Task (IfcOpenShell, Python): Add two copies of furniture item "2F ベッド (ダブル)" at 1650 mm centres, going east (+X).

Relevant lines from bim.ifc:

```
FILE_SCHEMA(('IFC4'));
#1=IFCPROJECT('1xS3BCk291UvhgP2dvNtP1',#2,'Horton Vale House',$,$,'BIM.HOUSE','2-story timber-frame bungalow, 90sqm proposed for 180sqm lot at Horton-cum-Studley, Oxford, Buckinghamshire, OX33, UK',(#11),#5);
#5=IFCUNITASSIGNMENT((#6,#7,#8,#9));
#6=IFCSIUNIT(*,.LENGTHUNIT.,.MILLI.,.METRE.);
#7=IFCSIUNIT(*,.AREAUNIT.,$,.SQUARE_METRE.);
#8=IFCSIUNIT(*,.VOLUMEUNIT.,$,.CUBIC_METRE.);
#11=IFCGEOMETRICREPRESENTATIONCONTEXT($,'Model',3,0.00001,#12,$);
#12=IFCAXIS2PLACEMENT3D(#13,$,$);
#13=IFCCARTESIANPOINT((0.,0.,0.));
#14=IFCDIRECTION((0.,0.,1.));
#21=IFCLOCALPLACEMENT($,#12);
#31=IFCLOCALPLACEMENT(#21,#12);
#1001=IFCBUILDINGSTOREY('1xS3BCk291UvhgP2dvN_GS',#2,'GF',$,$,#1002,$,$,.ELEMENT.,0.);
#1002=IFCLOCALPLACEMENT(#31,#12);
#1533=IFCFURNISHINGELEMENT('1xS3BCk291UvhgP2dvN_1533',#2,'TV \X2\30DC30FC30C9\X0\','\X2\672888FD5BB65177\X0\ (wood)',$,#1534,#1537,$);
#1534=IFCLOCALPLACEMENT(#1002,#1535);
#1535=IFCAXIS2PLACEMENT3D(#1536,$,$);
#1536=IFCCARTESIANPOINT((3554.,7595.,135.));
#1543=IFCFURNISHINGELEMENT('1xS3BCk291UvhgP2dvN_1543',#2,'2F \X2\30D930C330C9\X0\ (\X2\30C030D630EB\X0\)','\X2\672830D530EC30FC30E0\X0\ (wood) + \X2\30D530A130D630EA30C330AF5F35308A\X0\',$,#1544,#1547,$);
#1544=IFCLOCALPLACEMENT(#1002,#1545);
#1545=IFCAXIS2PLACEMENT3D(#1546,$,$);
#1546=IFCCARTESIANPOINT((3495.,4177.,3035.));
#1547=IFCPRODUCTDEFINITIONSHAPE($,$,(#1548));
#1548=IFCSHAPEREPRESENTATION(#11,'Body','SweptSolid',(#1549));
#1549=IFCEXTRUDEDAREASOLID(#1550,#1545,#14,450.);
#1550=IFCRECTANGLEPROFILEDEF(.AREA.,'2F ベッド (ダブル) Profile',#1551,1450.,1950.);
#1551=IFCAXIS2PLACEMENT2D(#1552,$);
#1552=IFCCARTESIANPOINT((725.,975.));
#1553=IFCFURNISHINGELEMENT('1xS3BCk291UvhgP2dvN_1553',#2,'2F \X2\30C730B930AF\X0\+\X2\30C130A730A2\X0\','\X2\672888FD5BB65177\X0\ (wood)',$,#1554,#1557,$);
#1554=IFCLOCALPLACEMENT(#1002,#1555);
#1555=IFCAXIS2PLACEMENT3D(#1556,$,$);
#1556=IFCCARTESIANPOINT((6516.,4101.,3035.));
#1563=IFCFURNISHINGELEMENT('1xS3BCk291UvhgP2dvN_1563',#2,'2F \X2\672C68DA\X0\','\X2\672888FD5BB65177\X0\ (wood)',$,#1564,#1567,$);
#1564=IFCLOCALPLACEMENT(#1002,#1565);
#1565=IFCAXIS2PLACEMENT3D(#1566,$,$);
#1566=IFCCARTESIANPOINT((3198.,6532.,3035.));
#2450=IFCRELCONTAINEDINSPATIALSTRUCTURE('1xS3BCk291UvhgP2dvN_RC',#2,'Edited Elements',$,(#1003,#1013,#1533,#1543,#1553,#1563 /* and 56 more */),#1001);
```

```python
import numpy as np
import ifcopenshell
import ifcopenshell.api.geometry
import ifcopenshell.api.root
import ifcopenshell.util.element
import ifcopenshell.util.placement

model = ifcopenshell.open("bim.ifc")


def reuse_history(source, copy):
    """copy_class also copies each property set's owner history, people and application; keep the originals."""
    for rel in copy.IsDefinedBy:
        if rel.is_a("IfcRelDefinesByProperties") and (history := rel.RelatingPropertyDefinition.OwnerHistory):
            rel.RelatingPropertyDefinition.OwnerHistory = source.OwnerHistory
            ifcopenshell.util.element.remove_deep2(model, history)


source = model.by_guid("1xS3BCk291UvhgP2dvN_1543")
base = ifcopenshell.util.placement.get_local_placement(source.ObjectPlacement)
step = np.array([1.0, 0.0, 0.0]) * 1650.0

for i in range(1, 3):
    copy = ifcopenshell.api.root.copy_class(model, product=source)
    copy.Representation = ifcopenshell.util.element.copy_deep(
        model, source.Representation, exclude=["IfcGeometricRepresentationContext", "IfcRepresentationMap"]
    )
    reuse_history(source, copy)
    matrix = base.copy()
    matrix[:3, 3] += i * step
    print("added at", matrix[:3, 3].round(3) + 0.0)
    ifcopenshell.api.geometry.edit_object_placement(model, product=copy, matrix=matrix, is_si=False)

model.write("bim_updated.ifc")
```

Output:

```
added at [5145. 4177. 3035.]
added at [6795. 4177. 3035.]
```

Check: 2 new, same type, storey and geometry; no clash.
